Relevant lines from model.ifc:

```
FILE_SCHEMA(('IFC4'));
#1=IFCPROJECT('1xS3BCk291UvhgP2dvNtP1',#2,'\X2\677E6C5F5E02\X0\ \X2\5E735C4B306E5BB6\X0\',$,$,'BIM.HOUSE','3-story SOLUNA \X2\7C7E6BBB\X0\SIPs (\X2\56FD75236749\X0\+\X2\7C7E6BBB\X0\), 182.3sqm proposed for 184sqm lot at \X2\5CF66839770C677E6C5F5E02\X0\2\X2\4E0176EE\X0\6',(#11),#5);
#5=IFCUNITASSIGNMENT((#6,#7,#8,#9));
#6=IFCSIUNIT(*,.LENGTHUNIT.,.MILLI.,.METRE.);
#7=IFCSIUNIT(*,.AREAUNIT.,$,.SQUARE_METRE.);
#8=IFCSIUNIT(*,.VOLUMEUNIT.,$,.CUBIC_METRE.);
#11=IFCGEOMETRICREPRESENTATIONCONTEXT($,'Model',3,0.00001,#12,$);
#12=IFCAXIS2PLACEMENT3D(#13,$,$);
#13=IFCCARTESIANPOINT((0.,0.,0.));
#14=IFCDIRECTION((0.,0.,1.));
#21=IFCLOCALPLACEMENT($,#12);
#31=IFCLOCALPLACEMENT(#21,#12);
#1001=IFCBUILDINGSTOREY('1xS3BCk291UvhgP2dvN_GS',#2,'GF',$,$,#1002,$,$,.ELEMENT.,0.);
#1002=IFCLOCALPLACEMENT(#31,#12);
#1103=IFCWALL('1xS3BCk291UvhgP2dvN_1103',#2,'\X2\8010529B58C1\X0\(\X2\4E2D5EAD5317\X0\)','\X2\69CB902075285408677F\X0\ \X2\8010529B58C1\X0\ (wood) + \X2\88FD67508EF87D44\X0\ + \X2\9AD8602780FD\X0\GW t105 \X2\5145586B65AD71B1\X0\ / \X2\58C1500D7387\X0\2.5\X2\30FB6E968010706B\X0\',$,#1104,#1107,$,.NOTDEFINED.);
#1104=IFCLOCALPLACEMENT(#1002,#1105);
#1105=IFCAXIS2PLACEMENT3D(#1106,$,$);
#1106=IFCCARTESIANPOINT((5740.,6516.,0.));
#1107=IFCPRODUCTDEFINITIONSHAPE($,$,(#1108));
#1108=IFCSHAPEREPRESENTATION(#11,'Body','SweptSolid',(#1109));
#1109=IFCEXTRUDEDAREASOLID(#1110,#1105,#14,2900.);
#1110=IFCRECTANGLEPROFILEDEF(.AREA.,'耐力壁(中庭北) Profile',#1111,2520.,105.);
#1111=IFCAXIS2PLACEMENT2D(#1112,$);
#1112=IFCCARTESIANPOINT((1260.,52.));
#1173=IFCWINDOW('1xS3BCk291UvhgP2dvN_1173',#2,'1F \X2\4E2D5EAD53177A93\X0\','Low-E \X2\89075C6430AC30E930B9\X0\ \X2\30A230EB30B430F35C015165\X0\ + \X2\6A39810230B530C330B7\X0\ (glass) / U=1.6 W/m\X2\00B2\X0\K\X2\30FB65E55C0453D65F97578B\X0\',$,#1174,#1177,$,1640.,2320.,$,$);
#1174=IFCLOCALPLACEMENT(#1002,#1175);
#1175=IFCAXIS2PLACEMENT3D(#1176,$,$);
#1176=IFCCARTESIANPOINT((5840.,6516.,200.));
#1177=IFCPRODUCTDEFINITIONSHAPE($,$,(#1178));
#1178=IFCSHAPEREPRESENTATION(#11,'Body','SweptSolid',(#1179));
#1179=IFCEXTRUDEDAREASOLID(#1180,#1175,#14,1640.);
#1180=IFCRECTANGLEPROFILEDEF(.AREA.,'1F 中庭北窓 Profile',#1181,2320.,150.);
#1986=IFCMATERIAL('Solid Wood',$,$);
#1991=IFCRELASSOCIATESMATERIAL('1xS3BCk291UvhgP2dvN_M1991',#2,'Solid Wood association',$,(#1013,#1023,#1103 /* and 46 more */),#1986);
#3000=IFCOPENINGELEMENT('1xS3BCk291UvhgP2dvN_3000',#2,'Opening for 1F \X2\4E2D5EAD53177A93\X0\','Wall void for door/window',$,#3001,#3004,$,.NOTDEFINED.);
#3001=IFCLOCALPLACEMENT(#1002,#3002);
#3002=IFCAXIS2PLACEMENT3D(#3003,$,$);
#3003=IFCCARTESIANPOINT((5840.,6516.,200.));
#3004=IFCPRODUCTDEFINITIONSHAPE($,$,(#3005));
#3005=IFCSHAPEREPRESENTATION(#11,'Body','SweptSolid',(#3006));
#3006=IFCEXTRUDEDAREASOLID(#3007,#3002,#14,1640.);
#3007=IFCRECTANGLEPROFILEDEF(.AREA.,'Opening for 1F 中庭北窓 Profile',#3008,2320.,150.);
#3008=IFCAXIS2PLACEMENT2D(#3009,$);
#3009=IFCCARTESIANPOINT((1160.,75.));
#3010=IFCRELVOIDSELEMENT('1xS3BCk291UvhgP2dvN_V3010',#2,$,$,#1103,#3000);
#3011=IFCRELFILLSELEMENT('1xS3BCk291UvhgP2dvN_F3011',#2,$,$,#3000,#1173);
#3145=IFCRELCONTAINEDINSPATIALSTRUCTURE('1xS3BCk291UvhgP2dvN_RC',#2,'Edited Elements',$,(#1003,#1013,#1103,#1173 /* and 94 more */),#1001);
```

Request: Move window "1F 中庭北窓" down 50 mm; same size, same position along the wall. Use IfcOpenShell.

```python
import numpy as np
import ifcopenshell
import ifcopenshell.api.geometry
import ifcopenshell.util.placement
import ifcopenshell.util.unit

model = ifcopenshell.open("model.ifc")
unit_scale = ifcopenshell.util.unit.calculate_unit_scale(model)

window = model.by_guid("1xS3BCk291UvhgP2dvN_1173")
opening = window.FillsVoids[0].RelatingOpeningElement
dz = -50.0

shift = np.array([0.0, 0.0, dz])
# The window is not placed relative to its opening, so move both.
for product in (opening, window):
    matrix = ifcopenshell.util.placement.get_local_placement(product.ObjectPlacement)
    matrix[:3, 3] += shift
    ifcopenshell.api.geometry.edit_object_placement(model, product=product, matrix=matrix, is_si=False)

print(f"moved by {dz * unit_scale:+.3f} m")

model.write("model_rev.ifc")
```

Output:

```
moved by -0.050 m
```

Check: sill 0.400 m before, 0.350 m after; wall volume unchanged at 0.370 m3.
